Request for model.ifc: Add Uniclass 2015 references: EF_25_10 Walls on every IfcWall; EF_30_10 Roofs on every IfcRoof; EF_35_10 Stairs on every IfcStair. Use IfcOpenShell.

First a look at what the model holds.

```python
import ifcopenshell

model = ifcopenshell.open("model.ifc")
print(model.schema)
print("classifications:", [c.Name for c in model.by_type("IfcClassification")])
for ifc_class in ("IfcDoor", "IfcRoof", "IfcStair", "IfcWall", "IfcWindow"):
    print(ifc_class, len(model.by_type(ifc_class)))
```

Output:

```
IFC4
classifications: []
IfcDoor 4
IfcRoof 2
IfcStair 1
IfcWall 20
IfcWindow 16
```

```python
import ifcopenshell
import ifcopenshell.api.classification

model = ifcopenshell.open("model.ifc")

system = ifcopenshell.api.classification.add_classification(model, classification="Uniclass 2015")

codes = {
    "IfcWall": ("EF_25_10", "Walls"),
    "IfcRoof": ("EF_30_10", "Roofs"),
    "IfcStair": ("EF_35_10", "Stairs"),
}
for ifc_class, (code, name) in codes.items():
    products = model.by_type(ifc_class)
    ifcopenshell.api.classification.add_reference(
        model, products=products, classification=system, identification=code, name=name
    )
    print(code, len(products))

model.write("model_rev.ifc")
```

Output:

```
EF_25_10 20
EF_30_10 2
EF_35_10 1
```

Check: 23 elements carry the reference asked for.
